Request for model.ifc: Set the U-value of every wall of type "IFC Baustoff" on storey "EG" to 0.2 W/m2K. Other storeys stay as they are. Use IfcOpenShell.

First a look at what the model holds.

```python
import ifcopenshell
import ifcopenshell.util.element

model = ifcopenshell.open("model.ifc")
print(model.schema)
storey = next(s for s in model.by_type("IfcBuildingStorey") if s.Name == "EG")
walls = [e for e in ifcopenshell.util.element.get_decomposition(storey) if e.is_a("IfcWall")]
seen = {}
for e in walls:
    element_type = ifcopenshell.util.element.get_type(e)
    key = (element_type.Name if element_type != e and element_type else None, ifcopenshell.util.element.get_pset(e, "Pset_WallCommon", "ThermalTransmittance"))
    seen[key] = seen.get(key, 0) + 1
for (name, value), count in sorted(seen.items(), key=str):
    print(count, "x", name, "|", value)
```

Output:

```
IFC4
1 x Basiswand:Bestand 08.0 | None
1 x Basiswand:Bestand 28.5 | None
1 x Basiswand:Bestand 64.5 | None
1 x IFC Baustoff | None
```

```python
import ifcopenshell
import ifcopenshell.api.pset
import ifcopenshell.util.element

model = ifcopenshell.open("model.ifc")

storey = next(s for s in model.by_type("IfcBuildingStorey") if s.Name == "EG")
walls = [e for e in ifcopenshell.util.element.get_decomposition(storey) if e.is_a("IfcWall")]

count = 0
for e in walls:
    element_type = ifcopenshell.util.element.get_type(e)
    if element_type in (None, e) or element_type.Name != "IFC Baustoff":
        continue
    # add_pset returns the element's existing set when there is one.
    pset = ifcopenshell.api.pset.add_pset(model, product=e, name="Pset_WallCommon")
    ifcopenshell.api.pset.edit_pset(model, pset=pset, properties={"ThermalTransmittance": 0.2})
    count += 1

print(count, "walls updated")

model.write("model_rev.ifc")
```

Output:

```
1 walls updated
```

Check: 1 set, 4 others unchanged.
